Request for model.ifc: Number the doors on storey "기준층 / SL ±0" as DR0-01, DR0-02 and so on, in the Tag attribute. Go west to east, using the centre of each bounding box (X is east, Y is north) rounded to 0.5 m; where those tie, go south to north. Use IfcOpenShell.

First a look at what the model holds.

```python
import ifcopenshell
import ifcopenshell.util.element
import ifcopenshell.util.placement

model = ifcopenshell.open("model.ifc")
print(model.schema)
storey = next(s for s in model.by_type("IfcBuildingStorey") if s.Name == "기준층 / SL ±0")
doors = [e for e in ifcopenshell.util.element.get_decomposition(storey) if e.is_a("IfcDoor")]
for e in sorted(doors, key=lambda e: e.id()):
    origin = ifcopenshell.util.placement.get_local_placement(e.ObjectPlacement)[:3, 3]
    print(e.id(), e.Tag, e.Name, origin.round(2) + 0.0, sep=" | ")
```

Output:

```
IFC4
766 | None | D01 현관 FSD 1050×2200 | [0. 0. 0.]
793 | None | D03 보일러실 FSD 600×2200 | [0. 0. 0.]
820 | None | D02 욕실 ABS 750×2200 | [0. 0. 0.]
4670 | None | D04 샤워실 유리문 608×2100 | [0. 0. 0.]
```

```python
import ifcopenshell
import ifcopenshell.geom
import ifcopenshell.util.element
import ifcopenshell.util.shape

model = ifcopenshell.open("model.ifc")
settings = ifcopenshell.geom.settings()
settings.set("use-world-coords", True)


def centre(element):
    shape = ifcopenshell.geom.create_shape(settings, element)
    return ifcopenshell.util.shape.get_bbox_centroid(shape.geometry)


storey = next(s for s in model.by_type("IfcBuildingStorey") if s.Name == "기준층 / SL ±0")
doors = [e for e in ifcopenshell.util.element.get_decomposition(storey) if e.is_a("IfcDoor")]

# Insertion points can sit at a corner or the storey origin, so sort by the geometry (in metres).
centres = {e: centre(e) for e in doors}
doors.sort(key=lambda e: (round(centres[e][0] / 0.5), centres[e][1]))

for i, e in enumerate(doors, start=1):
    number = f"DR0-{i:02d}"
    e.Tag = number
    print(e.id(), number)

model.write("model-out.ifc")
```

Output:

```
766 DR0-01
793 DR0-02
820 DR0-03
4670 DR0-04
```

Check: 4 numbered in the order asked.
